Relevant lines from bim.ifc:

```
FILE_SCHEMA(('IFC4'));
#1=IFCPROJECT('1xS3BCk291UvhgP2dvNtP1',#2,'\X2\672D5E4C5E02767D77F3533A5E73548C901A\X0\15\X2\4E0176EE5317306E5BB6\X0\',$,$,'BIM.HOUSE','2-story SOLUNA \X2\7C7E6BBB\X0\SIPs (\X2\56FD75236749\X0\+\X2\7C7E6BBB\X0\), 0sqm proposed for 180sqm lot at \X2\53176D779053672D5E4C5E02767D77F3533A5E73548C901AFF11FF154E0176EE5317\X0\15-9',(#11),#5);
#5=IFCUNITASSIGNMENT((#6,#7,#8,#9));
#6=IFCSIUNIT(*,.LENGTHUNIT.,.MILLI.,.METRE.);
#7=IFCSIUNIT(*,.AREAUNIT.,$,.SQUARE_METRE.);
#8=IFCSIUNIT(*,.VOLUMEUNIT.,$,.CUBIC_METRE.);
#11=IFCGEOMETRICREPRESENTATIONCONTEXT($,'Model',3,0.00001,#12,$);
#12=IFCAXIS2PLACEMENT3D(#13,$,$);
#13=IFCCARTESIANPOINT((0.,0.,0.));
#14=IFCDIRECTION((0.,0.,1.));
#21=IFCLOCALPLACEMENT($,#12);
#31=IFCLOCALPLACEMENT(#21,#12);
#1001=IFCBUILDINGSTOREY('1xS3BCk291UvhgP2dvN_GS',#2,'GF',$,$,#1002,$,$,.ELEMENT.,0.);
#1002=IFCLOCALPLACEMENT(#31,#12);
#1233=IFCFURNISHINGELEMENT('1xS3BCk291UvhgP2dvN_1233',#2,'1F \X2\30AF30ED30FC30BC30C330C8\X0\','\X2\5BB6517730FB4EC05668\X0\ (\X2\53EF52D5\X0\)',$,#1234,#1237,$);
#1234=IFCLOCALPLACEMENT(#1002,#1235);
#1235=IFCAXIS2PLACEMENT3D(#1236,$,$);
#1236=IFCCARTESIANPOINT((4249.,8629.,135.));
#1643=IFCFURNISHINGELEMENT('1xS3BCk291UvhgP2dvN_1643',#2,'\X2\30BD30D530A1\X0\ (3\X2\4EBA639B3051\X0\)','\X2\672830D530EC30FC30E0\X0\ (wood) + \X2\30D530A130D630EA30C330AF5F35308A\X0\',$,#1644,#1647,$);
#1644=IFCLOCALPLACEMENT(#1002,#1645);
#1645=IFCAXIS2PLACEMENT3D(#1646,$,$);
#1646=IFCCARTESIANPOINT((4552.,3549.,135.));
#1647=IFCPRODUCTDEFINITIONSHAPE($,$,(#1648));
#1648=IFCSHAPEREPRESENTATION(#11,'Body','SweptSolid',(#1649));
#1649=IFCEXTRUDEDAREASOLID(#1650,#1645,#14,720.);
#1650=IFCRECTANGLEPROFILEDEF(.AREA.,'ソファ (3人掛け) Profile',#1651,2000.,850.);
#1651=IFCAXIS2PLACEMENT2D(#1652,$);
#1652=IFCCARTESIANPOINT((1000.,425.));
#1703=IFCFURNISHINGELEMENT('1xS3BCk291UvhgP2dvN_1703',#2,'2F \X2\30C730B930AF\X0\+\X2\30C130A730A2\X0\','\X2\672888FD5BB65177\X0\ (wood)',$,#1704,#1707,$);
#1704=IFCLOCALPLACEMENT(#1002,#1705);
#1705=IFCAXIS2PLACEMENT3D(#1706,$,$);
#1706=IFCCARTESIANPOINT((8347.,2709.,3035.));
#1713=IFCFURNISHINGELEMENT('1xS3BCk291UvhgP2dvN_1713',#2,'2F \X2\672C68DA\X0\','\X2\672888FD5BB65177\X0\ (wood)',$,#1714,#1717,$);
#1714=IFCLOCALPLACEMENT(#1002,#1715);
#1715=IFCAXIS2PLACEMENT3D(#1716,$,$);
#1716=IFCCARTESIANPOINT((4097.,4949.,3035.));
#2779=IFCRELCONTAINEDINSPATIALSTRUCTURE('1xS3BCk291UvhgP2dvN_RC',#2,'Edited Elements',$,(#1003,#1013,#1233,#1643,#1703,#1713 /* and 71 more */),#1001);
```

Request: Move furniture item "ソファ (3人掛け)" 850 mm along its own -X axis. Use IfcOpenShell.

```python
import ifcopenshell
import ifcopenshell.api.geometry
import ifcopenshell.util.placement
import ifcopenshell.util.unit

model = ifcopenshell.open("bim.ifc")
unit_scale = ifcopenshell.util.unit.calculate_unit_scale(model)

item = model.by_guid("1xS3BCk291UvhgP2dvN_1643")
matrix = ifcopenshell.util.placement.get_local_placement(item.ObjectPlacement)
matrix[:3, 3] -= matrix[:3, 0] * 0.85 / unit_scale
ifcopenshell.api.geometry.edit_object_placement(model, product=item, matrix=matrix, is_si=False)

print(ifcopenshell.util.placement.get_local_placement(item.ObjectPlacement).round(3) + 0.0)

model.write("bim_edited.ifc")
```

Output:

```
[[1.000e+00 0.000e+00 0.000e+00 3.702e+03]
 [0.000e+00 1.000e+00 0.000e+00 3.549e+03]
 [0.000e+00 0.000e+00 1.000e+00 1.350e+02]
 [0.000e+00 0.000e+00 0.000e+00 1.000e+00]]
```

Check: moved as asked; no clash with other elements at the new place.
